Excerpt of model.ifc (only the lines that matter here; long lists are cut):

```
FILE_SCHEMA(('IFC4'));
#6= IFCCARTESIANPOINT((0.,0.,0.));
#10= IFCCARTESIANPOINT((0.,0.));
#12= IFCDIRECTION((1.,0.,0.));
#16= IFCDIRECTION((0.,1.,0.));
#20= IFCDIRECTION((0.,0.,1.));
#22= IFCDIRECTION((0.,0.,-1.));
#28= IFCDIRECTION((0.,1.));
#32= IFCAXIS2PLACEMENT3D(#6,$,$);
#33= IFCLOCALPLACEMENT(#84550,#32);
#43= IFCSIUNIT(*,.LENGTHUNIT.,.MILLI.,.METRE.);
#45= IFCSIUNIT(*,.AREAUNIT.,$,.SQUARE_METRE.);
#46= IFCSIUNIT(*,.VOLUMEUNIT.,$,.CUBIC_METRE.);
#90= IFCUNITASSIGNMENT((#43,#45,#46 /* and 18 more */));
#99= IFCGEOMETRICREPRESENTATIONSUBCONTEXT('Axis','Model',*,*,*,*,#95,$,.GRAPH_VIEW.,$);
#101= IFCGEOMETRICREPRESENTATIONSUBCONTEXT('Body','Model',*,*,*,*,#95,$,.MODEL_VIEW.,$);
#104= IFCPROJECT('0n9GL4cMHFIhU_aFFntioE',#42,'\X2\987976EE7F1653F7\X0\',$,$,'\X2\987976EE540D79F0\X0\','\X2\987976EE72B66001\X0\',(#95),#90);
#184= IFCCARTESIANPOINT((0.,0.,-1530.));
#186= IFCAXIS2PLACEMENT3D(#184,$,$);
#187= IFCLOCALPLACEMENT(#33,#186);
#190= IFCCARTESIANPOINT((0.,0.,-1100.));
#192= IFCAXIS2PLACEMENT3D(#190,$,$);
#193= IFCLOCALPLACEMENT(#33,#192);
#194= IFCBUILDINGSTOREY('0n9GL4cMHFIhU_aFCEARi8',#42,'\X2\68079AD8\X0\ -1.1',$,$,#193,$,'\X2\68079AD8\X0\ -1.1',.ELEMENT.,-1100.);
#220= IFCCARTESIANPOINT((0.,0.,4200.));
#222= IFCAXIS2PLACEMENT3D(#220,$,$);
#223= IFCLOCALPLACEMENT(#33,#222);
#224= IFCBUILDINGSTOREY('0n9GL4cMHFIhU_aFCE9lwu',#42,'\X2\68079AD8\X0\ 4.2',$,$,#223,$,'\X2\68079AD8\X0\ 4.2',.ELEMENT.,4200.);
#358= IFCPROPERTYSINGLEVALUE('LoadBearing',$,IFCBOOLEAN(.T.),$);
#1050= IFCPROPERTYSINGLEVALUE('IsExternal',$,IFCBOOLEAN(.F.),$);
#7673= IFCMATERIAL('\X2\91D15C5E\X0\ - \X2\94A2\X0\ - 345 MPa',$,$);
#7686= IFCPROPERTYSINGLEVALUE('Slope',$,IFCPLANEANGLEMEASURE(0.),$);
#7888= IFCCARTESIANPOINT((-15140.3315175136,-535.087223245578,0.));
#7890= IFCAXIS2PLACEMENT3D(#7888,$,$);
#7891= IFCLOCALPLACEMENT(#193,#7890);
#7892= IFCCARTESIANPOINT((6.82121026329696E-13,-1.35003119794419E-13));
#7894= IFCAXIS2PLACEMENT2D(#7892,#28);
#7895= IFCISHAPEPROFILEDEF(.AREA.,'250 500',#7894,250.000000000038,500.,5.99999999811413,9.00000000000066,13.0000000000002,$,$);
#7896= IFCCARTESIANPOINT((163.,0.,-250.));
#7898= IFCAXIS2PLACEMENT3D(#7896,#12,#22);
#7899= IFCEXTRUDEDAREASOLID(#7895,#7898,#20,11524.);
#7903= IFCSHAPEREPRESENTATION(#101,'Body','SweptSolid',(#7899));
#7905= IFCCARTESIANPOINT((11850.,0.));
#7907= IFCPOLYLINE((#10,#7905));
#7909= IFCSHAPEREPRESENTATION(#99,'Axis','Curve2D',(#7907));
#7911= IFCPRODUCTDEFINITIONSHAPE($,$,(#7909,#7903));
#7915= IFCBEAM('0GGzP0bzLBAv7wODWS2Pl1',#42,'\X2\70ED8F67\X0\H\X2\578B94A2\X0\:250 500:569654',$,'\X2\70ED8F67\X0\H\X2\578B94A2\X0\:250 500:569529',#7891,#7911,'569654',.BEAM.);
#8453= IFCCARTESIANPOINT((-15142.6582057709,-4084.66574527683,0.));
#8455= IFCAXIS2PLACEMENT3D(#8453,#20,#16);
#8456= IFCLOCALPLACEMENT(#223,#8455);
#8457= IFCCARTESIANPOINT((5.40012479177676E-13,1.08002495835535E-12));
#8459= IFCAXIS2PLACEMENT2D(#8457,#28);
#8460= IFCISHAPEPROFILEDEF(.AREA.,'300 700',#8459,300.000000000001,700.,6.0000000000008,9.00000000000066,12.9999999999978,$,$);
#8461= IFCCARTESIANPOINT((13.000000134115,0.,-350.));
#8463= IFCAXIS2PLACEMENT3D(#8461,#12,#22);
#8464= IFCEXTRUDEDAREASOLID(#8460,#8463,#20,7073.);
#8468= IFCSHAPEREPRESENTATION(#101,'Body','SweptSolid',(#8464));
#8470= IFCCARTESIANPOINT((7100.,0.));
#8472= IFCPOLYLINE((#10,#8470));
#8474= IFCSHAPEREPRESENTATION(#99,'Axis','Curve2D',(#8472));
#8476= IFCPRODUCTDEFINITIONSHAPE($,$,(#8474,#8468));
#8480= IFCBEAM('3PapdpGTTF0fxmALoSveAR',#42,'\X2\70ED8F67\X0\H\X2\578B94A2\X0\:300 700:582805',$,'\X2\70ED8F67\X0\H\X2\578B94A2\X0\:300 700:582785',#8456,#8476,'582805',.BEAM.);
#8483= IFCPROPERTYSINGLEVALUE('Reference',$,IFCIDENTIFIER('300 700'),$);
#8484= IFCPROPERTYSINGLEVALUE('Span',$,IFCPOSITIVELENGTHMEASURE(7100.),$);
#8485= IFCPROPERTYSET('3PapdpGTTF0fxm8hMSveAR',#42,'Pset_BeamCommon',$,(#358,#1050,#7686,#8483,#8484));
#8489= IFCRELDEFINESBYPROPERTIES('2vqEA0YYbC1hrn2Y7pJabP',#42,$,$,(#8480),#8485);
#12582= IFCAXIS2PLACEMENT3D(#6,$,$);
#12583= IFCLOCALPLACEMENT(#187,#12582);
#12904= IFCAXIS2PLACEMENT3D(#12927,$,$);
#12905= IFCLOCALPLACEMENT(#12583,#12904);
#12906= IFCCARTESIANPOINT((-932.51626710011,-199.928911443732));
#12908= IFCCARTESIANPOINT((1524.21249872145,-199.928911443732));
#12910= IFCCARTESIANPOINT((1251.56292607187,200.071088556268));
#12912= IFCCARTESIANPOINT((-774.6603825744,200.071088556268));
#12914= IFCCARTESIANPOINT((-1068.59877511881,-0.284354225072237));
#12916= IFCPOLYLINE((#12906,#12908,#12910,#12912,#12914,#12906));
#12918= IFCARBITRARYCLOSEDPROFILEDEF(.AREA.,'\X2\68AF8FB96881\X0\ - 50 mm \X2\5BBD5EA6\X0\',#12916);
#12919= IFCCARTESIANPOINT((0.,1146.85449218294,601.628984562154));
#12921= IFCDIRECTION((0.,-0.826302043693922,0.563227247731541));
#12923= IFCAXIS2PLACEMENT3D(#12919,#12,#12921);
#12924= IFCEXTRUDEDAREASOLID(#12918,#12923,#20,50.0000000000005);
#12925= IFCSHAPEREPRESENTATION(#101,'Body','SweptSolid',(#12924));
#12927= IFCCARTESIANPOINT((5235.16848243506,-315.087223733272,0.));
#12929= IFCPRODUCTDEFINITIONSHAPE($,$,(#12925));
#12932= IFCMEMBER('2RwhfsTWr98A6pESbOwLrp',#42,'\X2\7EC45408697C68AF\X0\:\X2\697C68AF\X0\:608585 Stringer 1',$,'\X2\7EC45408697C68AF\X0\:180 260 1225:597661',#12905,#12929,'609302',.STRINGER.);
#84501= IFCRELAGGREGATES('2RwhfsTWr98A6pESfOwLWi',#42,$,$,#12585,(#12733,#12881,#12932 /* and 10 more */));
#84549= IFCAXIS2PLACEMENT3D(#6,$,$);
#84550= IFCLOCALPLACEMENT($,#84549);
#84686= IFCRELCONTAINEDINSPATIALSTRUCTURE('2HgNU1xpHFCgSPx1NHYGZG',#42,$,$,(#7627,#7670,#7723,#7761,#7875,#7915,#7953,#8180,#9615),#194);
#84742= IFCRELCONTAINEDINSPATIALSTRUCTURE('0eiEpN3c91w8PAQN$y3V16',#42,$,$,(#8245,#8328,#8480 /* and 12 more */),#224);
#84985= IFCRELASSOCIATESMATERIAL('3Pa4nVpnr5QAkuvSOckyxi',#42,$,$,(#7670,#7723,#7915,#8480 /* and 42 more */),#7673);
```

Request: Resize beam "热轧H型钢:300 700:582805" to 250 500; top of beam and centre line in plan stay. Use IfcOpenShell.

```python
import ifcopenshell
import ifcopenshell.api.pset
import ifcopenshell.util.element
import ifcopenshell.util.representation

model = ifcopenshell.open("model.ifc")

member = model.by_id(8480)
source = next(p for p in model.by_type("IfcIShapeProfileDef") if p.ProfileName == "250 500")

body = ifcopenshell.util.representation.get_representation(member, "Model", "Body")
solid = body.Items[0]
old_profile = solid.SweptArea

# Copy the section's sizes but keep this member's own profile position.
profile = ifcopenshell.util.element.copy(model, source)
# Profiles are centred, so shift by half the change in depth to hold the top.
shift = (old_profile.OverallDepth - profile.OverallDepth) / 2
x, y = old_profile.Position.Location.Coordinates
up = (-1.0, 0.0)  # upwards, in the solid's own plane
location = model.createIfcCartesianPoint((x + up[0] * shift, y + up[1] * shift))
profile.Position = model.createIfcAxis2Placement2D(location, old_profile.Position.RefDirection)
solid.SweptArea = profile
if not model.get_total_inverses(old_profile):
    ifcopenshell.util.element.remove_deep2(model, old_profile)
member.Name = member.Name.replace("300 700", "250 500")
member.ObjectType = member.ObjectType.replace("300 700", "250 500")
pset = model.by_id(ifcopenshell.util.element.get_pset(member, "Pset_BeamCommon", should_inherit=False)["id"])
ifcopenshell.api.pset.edit_pset(model, pset=pset, properties={"Reference": "250 500"})

print(solid.SweptArea)

model.write("model-out.ifc")
```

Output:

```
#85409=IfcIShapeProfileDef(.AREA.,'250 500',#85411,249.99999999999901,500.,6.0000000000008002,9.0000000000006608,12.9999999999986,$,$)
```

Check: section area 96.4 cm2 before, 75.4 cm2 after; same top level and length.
